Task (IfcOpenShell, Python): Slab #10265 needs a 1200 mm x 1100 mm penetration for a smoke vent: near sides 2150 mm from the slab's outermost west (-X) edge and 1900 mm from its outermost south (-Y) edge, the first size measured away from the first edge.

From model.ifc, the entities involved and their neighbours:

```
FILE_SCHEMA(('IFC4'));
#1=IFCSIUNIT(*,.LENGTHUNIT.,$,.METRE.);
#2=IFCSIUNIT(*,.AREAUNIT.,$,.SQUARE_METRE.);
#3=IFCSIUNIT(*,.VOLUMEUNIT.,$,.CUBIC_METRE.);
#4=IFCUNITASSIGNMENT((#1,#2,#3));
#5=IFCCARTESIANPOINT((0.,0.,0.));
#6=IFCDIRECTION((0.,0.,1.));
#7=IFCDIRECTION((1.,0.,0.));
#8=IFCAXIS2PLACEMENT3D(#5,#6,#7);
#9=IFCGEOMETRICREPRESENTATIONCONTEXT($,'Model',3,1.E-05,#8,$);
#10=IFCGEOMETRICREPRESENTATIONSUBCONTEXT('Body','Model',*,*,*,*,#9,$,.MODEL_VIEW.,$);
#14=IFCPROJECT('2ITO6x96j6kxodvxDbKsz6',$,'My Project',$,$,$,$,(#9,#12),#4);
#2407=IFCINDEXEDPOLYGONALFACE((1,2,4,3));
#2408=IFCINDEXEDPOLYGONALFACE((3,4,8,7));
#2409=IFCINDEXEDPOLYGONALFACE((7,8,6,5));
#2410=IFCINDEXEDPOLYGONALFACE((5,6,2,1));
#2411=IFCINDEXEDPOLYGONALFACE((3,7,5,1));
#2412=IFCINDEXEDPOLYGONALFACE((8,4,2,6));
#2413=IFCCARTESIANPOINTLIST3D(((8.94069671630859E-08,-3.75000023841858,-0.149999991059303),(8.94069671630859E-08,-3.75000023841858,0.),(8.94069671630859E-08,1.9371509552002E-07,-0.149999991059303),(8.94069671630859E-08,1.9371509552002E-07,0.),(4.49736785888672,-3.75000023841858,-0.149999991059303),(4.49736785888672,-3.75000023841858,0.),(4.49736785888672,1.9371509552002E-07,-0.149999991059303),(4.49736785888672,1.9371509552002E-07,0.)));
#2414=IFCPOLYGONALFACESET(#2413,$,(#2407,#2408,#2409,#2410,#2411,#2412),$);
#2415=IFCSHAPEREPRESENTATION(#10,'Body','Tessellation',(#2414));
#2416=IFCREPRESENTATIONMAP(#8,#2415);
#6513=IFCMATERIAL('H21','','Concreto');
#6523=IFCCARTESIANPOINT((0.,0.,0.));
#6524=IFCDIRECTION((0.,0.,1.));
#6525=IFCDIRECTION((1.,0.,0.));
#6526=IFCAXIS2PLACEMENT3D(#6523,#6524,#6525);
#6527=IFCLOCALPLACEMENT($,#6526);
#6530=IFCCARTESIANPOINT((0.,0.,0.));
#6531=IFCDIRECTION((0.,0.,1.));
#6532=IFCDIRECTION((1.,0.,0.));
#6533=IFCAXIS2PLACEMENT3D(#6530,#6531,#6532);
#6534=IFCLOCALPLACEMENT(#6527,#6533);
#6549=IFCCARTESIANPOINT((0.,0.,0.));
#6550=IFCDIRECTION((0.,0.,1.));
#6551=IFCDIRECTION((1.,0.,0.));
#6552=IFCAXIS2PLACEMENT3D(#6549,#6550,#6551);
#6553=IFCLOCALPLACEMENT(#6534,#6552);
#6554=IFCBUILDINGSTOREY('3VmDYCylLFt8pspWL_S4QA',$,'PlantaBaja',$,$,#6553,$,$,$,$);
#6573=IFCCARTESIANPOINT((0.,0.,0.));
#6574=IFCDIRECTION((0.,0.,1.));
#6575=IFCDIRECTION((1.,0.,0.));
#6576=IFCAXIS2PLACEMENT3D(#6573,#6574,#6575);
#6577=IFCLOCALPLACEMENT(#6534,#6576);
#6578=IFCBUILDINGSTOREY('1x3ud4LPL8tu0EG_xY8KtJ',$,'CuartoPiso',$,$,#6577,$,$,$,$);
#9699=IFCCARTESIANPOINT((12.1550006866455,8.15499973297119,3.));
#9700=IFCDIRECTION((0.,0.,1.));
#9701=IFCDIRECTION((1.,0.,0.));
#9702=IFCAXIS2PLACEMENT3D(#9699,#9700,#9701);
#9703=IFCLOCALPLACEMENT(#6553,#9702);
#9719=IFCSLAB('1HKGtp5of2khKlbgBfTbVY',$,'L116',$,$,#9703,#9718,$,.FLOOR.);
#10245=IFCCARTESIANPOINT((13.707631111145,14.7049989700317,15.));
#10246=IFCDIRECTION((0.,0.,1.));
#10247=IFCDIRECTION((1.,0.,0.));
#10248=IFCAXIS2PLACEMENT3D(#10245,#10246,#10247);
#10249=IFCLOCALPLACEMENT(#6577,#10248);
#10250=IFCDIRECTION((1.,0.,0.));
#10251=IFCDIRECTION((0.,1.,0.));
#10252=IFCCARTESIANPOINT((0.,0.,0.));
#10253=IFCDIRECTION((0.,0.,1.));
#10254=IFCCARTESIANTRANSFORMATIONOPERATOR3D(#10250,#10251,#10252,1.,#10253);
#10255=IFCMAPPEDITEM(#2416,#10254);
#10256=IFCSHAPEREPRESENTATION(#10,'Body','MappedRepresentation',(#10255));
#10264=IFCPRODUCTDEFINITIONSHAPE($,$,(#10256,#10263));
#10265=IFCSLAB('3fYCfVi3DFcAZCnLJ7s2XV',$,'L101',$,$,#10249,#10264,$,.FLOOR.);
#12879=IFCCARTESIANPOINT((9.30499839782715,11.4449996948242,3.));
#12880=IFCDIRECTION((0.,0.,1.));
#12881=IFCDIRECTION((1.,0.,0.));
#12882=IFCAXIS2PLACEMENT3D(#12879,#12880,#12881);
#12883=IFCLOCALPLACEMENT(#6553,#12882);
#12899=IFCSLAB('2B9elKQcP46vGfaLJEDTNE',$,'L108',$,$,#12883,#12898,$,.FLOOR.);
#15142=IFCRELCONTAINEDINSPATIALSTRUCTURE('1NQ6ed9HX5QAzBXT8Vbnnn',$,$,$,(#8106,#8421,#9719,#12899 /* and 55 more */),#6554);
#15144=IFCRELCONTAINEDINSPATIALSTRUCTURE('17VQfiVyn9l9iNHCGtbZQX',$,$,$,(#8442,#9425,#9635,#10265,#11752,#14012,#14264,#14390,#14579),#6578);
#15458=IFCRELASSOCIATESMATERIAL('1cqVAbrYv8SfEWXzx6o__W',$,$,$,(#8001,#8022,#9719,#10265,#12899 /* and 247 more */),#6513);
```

```python
import numpy as np
import ifcopenshell
import ifcopenshell.api.feature
import ifcopenshell.api.geometry
import ifcopenshell.api.root
import ifcopenshell.geom
import ifcopenshell.util.placement
import ifcopenshell.util.representation
import ifcopenshell.util.shape
import ifcopenshell.util.unit

model = ifcopenshell.open("model.ifc")
unit_scale = ifcopenshell.util.unit.calculate_unit_scale(model)
settings = ifcopenshell.geom.settings()


def volume(element):
    """Net volume in cubic metres, openings subtracted."""
    shape = ifcopenshell.geom.create_shape(settings, element)
    return ifcopenshell.util.shape.get_volume(shape.geometry)


slab = model.by_guid("3fYCfVi3DFcAZCnLJ7s2XV")
before = volume(slab)

# Extent in the slab's own axes, in metres. The edges named are its -X and -Y sides.
slab_shape = ifcopenshell.geom.create_shape(settings, slab)
vertices = ifcopenshell.util.shape.get_vertices(slab_shape.geometry)
x_min, y_min, bottom = vertices.min(axis=0)
top = vertices[:, 2].max()

opening = ifcopenshell.api.root.create_entity(model, ifc_class="IfcOpeningElement", name="Smoke vent opening", predefined_type="OPENING")
context = ifcopenshell.util.representation.get_context(model, "Model", "Body", "MODEL_VIEW")
width, depth = 1.2, 1.1
outline = [(0.0, 0.0), (width, 0.0), (width, depth), (0.0, depth), (0.0, 0.0)]
# Overshoot both faces by 50 mm so the cut is clean.
shape = ifcopenshell.api.geometry.add_slab_representation(
    model, context=context, depth=top - bottom + 0.1, polyline=outline
)
ifcopenshell.api.geometry.assign_representation(model, product=opening, representation=shape)

matrix = ifcopenshell.util.placement.get_local_placement(slab.ObjectPlacement)
matrix[:, 3] = matrix @ np.append(np.array([x_min + 2.15, y_min + 1.9, bottom - 0.05]) / unit_scale, 1.0)
ifcopenshell.api.geometry.edit_object_placement(model, product=opening, matrix=matrix, is_si=False)
ifcopenshell.api.feature.add_feature(model, feature=opening, element=slab)

after = volume(slab)

print(f"slab volume {before:.3f} -> {after:.3f} m3")

model.write("model_updated.ifc")
```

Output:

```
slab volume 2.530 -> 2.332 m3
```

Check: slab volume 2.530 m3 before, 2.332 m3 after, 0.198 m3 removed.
